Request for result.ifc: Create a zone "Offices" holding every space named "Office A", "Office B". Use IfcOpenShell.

First a look at what the model holds.

```python
import ifcopenshell

model = ifcopenshell.open("result.ifc")
print(model.schema)
seen = {}
for space in model.by_type("IfcSpace"):
    seen[space.Name] = seen.get(space.Name, 0) + 1
for name, count in sorted(seen.items(), key=str):
    print(count, "x", name)
print("zones:", [z.Name for z in model.by_type("IfcZone")][:20])
```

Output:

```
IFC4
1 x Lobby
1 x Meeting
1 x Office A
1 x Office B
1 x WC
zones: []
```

```python
import ifcopenshell
import ifcopenshell.api.group
import ifcopenshell.api.root

model = ifcopenshell.open("result.ifc")

names = {"Office A", "Office B"}
spaces = [s for s in model.by_type("IfcSpace") if s.Name in names]

zone = ifcopenshell.api.root.create_entity(model, ifc_class="IfcZone", name="Offices")
ifcopenshell.api.group.assign_group(model, products=spaces, group=zone)
print(len(spaces), "spaces in", zone.Name)

model.write("result_v2.ifc")
```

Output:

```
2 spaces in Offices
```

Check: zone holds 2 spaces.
